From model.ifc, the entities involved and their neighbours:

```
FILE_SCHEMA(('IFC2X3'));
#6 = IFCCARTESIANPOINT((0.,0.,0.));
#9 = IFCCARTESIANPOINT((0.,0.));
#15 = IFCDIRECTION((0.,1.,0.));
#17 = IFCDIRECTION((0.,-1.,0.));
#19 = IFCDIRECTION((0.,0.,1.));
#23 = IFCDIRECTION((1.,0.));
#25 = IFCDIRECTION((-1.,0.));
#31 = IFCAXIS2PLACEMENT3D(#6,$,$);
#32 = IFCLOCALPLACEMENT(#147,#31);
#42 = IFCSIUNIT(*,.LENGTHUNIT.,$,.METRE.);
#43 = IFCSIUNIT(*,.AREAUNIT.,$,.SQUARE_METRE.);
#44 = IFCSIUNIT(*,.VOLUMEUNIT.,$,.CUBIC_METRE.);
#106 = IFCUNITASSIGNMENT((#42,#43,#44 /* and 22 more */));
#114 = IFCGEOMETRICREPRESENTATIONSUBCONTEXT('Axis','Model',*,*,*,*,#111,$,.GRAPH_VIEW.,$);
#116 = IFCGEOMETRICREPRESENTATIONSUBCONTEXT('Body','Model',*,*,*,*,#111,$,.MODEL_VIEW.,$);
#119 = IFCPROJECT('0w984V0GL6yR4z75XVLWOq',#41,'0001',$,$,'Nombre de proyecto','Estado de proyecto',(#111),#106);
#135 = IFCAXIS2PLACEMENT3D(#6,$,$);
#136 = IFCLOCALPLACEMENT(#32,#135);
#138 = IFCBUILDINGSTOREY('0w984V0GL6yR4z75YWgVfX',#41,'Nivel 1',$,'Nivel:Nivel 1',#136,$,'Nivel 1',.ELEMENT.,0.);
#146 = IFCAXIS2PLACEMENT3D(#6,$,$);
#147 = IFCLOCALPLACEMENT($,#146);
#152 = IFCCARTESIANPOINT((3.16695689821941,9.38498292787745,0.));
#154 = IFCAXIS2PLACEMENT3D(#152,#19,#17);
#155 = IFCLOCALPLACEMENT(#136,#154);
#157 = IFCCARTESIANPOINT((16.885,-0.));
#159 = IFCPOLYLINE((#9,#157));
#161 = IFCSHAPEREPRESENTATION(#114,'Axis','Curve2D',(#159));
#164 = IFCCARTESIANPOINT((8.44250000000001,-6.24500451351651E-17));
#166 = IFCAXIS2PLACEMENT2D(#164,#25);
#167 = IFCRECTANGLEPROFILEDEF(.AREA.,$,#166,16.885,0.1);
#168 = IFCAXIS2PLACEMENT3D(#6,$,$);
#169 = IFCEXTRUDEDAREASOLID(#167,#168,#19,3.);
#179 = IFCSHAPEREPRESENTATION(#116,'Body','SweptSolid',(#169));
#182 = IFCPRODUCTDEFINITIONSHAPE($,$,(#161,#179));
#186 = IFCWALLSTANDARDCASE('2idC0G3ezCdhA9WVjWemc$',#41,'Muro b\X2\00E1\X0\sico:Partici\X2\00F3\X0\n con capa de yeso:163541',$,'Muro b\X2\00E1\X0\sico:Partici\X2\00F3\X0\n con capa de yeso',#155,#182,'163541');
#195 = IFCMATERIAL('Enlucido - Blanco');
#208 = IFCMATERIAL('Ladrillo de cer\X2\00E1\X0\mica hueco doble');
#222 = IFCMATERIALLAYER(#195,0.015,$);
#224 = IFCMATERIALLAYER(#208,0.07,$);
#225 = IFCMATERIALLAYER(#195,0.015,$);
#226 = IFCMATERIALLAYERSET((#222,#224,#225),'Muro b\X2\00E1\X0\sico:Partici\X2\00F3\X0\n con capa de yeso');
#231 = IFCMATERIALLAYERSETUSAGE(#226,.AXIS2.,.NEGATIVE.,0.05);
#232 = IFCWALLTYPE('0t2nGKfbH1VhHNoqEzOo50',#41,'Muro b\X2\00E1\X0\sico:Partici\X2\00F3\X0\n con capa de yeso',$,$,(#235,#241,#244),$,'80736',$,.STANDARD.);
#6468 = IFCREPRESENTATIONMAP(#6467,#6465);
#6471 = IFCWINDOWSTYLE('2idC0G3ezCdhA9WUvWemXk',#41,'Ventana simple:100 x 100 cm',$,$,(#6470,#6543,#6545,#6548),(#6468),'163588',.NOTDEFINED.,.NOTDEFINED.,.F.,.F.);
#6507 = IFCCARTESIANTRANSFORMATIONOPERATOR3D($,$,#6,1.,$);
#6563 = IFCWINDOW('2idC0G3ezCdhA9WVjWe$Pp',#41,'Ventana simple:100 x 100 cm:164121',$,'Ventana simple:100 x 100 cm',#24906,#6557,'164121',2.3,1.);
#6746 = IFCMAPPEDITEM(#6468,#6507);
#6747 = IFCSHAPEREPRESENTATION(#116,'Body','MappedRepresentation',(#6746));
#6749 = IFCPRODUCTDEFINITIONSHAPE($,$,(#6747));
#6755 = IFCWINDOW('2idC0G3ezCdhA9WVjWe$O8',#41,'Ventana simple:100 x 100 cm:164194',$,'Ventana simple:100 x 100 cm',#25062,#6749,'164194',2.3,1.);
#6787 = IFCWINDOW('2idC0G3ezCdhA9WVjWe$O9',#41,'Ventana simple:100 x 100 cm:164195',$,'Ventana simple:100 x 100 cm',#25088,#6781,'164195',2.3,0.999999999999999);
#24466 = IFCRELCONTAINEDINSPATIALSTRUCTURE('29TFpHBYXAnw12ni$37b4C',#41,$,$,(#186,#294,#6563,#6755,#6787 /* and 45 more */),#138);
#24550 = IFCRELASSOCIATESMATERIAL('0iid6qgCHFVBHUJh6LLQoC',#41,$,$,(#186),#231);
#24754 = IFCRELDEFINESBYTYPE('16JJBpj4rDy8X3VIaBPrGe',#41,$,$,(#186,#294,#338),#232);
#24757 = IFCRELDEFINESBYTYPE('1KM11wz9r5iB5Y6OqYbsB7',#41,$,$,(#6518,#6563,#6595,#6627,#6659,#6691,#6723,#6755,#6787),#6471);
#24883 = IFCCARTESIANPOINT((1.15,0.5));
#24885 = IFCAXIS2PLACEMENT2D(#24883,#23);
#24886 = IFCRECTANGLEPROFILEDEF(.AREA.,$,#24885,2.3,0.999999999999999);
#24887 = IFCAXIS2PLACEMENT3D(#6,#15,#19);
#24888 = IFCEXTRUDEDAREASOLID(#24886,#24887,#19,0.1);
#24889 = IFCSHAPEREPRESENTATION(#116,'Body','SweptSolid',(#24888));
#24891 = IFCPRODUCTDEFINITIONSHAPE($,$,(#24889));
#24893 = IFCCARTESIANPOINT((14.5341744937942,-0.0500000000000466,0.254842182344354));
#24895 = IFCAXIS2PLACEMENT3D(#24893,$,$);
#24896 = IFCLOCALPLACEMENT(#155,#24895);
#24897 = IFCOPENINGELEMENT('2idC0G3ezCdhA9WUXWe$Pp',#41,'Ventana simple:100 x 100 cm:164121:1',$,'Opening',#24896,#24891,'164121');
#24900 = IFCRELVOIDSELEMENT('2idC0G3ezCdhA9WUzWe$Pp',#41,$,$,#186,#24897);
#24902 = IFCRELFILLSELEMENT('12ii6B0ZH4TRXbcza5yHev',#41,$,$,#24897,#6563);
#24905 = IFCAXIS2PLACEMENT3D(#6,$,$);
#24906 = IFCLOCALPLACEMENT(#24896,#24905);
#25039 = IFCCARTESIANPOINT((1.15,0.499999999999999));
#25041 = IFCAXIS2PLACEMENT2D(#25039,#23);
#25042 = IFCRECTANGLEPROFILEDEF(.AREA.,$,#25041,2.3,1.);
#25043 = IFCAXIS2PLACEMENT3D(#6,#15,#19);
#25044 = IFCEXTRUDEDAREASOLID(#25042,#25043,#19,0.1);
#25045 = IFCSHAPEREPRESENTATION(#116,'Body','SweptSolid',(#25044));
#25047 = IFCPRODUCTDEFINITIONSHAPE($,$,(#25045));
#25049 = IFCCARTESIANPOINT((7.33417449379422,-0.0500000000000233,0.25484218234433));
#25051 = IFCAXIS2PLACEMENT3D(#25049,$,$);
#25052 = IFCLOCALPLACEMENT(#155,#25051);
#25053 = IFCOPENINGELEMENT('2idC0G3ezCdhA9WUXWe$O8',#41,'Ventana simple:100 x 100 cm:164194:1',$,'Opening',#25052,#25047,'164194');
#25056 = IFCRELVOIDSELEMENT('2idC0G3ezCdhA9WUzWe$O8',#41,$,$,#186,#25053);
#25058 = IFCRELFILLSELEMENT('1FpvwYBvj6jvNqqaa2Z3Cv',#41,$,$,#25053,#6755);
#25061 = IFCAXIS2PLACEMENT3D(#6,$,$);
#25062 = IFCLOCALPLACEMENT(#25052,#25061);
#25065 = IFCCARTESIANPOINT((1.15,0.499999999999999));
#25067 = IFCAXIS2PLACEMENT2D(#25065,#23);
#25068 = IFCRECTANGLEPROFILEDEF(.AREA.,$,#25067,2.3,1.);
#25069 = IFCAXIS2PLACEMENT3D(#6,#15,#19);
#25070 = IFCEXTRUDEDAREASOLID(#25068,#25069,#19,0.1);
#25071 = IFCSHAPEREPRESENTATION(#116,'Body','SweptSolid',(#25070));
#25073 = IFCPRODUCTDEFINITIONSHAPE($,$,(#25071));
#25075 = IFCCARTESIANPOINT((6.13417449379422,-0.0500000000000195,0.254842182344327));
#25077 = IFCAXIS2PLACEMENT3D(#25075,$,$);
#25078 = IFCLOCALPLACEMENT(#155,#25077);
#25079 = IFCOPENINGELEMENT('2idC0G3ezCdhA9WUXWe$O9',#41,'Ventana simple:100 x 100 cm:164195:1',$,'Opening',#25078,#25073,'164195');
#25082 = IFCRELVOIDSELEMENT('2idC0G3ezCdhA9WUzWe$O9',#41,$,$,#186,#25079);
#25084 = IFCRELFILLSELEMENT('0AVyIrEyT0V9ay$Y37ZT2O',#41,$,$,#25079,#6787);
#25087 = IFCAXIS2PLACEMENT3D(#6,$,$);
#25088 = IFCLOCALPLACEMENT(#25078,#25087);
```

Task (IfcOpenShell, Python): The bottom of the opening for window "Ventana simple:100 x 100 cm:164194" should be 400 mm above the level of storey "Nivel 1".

```python
import numpy as np
import ifcopenshell
import ifcopenshell.api.geometry
import ifcopenshell.geom
import ifcopenshell.util.element
import ifcopenshell.util.placement
import ifcopenshell.util.shape
import ifcopenshell.util.unit

model = ifcopenshell.open("model.ifc")
unit_scale = ifcopenshell.util.unit.calculate_unit_scale(model)

window = model.by_id(6755)
opening = window.FillsVoids[0].RelatingOpeningElement
storey = ifcopenshell.util.element.get_container(window, ifc_class="IfcBuildingStorey")
level = ifcopenshell.util.placement.get_local_placement(storey.ObjectPlacement)[2, 3]

# The opening's origin need not be at the sill, so measure its lowest point.
shape = ifcopenshell.geom.create_shape(ifcopenshell.geom.settings(), opening)
bottom = ifcopenshell.util.shape.get_shape_bottom_elevation(shape, shape.geometry) / unit_scale
dz = level + 0.4 / unit_scale - bottom

shift = np.array([0.0, 0.0, dz])
# The window is placed relative to its opening, so it follows when the opening moves.
matrix = ifcopenshell.util.placement.get_local_placement(opening.ObjectPlacement)
matrix[:3, 3] += shift
ifcopenshell.api.geometry.edit_object_placement(
    model, product=opening, matrix=matrix, is_si=False, should_transform_children=True
)

print(f"moved by {dz * unit_scale:+.3f} m")

model.write("model_edited.ifc")
```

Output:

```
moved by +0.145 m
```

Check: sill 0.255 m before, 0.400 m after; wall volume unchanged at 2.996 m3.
